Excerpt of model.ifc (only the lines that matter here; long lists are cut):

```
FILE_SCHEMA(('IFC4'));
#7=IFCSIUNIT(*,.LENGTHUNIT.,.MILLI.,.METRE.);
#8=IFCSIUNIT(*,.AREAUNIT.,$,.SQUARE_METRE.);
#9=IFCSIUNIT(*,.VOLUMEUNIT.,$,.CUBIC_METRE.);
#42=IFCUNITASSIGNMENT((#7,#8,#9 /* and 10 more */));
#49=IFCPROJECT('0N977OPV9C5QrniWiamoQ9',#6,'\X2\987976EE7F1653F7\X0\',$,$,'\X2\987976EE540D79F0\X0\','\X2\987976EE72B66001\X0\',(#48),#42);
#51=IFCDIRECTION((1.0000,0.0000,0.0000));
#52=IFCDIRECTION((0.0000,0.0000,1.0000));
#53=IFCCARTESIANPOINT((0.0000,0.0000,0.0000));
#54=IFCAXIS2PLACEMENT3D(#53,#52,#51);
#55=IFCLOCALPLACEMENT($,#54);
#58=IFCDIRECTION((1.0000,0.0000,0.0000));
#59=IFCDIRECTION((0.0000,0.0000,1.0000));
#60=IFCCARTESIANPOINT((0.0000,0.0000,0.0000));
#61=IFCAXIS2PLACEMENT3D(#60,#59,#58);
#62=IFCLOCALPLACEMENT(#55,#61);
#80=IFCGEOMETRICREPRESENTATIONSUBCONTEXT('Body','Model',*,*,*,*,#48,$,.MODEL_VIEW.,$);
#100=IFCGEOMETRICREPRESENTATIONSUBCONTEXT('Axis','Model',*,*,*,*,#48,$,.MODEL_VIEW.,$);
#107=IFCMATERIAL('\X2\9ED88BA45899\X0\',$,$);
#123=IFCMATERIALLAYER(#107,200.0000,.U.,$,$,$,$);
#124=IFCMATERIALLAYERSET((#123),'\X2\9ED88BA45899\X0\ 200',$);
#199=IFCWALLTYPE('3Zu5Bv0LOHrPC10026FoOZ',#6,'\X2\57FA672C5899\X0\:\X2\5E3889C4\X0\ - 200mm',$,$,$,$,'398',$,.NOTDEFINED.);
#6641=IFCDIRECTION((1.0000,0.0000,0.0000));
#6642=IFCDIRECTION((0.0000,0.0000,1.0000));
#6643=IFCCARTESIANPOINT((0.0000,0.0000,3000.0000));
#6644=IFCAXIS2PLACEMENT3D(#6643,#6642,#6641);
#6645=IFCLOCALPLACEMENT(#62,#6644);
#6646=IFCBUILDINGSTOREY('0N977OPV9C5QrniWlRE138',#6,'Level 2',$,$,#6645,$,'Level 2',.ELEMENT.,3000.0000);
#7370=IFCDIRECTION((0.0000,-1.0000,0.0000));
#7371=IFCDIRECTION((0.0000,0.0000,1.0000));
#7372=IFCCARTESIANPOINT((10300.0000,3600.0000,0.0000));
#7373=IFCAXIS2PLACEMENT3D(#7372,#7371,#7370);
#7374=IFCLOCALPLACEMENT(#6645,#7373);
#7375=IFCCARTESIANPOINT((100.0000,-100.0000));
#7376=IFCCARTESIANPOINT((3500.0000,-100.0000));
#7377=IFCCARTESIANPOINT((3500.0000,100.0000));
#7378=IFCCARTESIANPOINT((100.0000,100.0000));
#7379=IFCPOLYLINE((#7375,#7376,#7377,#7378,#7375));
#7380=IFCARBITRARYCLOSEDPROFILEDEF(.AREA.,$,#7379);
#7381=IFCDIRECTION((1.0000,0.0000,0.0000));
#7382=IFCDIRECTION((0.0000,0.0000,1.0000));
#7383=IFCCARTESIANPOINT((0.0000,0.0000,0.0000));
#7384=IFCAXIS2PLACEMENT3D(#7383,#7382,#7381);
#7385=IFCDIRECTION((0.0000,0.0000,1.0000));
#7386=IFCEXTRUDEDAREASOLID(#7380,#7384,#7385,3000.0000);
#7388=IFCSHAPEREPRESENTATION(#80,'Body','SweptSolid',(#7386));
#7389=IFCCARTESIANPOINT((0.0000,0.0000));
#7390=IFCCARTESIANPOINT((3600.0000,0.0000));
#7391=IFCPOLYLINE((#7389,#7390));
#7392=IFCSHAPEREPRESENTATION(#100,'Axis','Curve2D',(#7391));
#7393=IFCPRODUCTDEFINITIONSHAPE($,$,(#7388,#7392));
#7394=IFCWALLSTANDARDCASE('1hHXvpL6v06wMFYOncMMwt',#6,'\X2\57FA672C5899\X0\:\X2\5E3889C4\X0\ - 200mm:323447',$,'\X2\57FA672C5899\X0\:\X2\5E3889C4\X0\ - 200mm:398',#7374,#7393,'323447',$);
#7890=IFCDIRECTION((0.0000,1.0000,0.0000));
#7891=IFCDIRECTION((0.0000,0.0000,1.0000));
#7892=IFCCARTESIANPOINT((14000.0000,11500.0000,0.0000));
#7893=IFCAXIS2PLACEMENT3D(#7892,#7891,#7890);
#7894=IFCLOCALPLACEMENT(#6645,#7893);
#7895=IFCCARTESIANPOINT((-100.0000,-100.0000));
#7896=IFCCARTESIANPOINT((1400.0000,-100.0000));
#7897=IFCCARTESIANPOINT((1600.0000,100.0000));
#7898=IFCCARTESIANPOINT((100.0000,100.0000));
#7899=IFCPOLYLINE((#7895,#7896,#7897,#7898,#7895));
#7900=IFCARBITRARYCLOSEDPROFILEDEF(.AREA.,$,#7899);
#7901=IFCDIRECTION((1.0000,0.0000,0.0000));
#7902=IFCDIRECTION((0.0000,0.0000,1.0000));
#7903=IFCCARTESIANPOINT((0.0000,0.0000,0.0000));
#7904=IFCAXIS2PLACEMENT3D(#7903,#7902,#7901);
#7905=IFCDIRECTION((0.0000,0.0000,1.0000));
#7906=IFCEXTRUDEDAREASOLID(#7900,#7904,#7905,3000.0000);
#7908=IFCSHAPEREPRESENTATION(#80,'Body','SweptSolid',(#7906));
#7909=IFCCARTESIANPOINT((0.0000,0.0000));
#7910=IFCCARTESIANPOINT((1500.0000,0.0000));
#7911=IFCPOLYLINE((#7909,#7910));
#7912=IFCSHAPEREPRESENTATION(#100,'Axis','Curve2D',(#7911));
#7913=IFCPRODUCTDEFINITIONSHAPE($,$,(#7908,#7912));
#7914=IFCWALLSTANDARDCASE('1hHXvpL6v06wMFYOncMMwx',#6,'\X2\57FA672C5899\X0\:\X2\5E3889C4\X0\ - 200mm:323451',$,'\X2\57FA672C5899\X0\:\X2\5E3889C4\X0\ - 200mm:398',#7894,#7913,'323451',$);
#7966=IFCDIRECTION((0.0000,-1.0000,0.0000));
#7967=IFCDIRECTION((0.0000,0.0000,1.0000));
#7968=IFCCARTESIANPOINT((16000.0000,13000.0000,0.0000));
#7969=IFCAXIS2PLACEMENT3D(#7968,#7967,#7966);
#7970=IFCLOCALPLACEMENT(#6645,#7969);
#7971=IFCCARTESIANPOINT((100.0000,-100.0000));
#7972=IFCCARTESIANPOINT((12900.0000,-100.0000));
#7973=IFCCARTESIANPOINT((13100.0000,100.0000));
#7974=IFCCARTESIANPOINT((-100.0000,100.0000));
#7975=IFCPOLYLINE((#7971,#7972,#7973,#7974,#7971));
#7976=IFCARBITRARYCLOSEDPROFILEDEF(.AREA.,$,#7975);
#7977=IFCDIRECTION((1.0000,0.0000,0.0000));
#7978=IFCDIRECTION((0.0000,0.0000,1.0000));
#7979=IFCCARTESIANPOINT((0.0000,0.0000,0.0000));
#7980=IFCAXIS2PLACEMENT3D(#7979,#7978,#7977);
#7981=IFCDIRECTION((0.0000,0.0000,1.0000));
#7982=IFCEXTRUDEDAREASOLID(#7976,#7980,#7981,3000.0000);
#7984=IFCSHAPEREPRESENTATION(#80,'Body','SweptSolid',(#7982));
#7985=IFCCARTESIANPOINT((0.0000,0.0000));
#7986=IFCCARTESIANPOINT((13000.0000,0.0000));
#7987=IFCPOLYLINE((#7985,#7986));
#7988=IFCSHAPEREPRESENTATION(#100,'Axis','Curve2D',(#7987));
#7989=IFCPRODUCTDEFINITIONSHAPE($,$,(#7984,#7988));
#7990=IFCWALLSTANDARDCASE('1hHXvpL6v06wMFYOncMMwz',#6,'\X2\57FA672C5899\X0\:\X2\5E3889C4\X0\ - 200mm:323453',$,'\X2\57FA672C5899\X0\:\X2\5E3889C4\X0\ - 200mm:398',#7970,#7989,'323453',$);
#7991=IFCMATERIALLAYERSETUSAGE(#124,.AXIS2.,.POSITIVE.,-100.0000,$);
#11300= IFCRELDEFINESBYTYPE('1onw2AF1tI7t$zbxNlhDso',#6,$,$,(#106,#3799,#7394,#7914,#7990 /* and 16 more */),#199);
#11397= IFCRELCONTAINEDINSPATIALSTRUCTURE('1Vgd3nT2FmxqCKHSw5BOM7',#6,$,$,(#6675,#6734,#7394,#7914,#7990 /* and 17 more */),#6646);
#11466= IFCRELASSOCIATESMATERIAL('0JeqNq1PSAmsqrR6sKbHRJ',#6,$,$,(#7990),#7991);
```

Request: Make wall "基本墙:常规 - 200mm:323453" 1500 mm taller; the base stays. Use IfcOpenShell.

```python
import ifcopenshell
import ifcopenshell.geom
import ifcopenshell.util.representation
import ifcopenshell.util.shape
import ifcopenshell.util.unit

model = ifcopenshell.open("model.ifc")
unit_scale = ifcopenshell.util.unit.calculate_unit_scale(model)
settings = ifcopenshell.geom.settings()


def volume(element):
    """Net volume in cubic metres, openings subtracted."""
    shape = ifcopenshell.geom.create_shape(settings, element)
    return ifcopenshell.util.shape.get_volume(shape.geometry)


wall = model.by_guid("1hHXvpL6v06wMFYOncMMwz")
before = volume(wall)

body = ifcopenshell.util.representation.get_representation(wall, "Model", "Body")
solid = body.Items[0]
old_height = solid.Depth
solid.Depth += 1.5 / unit_scale
after = volume(wall)

print(f"height {old_height:g} -> {solid.Depth:g}, volume {before:.3f} -> {after:.3f} m3")

model.write("model-out.ifc")
```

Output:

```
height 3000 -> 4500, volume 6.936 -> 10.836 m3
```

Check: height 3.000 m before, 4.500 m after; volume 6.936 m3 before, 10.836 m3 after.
